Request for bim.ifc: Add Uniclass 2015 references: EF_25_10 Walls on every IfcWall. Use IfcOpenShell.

First a look at what the model holds.

```python
import ifcopenshell

model = ifcopenshell.open("bim.ifc")
print(model.schema)
print("classifications:", [c.Name for c in model.by_type("IfcClassification")])
for ifc_class in ("IfcDoor", "IfcRoof", "IfcStair", "IfcWall", "IfcWindow"):
    print(ifc_class, len(model.by_type(ifc_class)))
```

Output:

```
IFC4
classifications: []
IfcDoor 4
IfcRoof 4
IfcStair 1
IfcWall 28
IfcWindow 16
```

```python
import ifcopenshell
import ifcopenshell.api.classification

model = ifcopenshell.open("bim.ifc")

system = ifcopenshell.api.classification.add_classification(model, classification="Uniclass 2015")

codes = {
    "IfcWall": ("EF_25_10", "Walls"),
}
for ifc_class, (code, name) in codes.items():
    products = model.by_type(ifc_class)
    ifcopenshell.api.classification.add_reference(
        model, products=products, classification=system, identification=code, name=name
    )
    print(code, len(products))

model.write("bim_v2.ifc")
```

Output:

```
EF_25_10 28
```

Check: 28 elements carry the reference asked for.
